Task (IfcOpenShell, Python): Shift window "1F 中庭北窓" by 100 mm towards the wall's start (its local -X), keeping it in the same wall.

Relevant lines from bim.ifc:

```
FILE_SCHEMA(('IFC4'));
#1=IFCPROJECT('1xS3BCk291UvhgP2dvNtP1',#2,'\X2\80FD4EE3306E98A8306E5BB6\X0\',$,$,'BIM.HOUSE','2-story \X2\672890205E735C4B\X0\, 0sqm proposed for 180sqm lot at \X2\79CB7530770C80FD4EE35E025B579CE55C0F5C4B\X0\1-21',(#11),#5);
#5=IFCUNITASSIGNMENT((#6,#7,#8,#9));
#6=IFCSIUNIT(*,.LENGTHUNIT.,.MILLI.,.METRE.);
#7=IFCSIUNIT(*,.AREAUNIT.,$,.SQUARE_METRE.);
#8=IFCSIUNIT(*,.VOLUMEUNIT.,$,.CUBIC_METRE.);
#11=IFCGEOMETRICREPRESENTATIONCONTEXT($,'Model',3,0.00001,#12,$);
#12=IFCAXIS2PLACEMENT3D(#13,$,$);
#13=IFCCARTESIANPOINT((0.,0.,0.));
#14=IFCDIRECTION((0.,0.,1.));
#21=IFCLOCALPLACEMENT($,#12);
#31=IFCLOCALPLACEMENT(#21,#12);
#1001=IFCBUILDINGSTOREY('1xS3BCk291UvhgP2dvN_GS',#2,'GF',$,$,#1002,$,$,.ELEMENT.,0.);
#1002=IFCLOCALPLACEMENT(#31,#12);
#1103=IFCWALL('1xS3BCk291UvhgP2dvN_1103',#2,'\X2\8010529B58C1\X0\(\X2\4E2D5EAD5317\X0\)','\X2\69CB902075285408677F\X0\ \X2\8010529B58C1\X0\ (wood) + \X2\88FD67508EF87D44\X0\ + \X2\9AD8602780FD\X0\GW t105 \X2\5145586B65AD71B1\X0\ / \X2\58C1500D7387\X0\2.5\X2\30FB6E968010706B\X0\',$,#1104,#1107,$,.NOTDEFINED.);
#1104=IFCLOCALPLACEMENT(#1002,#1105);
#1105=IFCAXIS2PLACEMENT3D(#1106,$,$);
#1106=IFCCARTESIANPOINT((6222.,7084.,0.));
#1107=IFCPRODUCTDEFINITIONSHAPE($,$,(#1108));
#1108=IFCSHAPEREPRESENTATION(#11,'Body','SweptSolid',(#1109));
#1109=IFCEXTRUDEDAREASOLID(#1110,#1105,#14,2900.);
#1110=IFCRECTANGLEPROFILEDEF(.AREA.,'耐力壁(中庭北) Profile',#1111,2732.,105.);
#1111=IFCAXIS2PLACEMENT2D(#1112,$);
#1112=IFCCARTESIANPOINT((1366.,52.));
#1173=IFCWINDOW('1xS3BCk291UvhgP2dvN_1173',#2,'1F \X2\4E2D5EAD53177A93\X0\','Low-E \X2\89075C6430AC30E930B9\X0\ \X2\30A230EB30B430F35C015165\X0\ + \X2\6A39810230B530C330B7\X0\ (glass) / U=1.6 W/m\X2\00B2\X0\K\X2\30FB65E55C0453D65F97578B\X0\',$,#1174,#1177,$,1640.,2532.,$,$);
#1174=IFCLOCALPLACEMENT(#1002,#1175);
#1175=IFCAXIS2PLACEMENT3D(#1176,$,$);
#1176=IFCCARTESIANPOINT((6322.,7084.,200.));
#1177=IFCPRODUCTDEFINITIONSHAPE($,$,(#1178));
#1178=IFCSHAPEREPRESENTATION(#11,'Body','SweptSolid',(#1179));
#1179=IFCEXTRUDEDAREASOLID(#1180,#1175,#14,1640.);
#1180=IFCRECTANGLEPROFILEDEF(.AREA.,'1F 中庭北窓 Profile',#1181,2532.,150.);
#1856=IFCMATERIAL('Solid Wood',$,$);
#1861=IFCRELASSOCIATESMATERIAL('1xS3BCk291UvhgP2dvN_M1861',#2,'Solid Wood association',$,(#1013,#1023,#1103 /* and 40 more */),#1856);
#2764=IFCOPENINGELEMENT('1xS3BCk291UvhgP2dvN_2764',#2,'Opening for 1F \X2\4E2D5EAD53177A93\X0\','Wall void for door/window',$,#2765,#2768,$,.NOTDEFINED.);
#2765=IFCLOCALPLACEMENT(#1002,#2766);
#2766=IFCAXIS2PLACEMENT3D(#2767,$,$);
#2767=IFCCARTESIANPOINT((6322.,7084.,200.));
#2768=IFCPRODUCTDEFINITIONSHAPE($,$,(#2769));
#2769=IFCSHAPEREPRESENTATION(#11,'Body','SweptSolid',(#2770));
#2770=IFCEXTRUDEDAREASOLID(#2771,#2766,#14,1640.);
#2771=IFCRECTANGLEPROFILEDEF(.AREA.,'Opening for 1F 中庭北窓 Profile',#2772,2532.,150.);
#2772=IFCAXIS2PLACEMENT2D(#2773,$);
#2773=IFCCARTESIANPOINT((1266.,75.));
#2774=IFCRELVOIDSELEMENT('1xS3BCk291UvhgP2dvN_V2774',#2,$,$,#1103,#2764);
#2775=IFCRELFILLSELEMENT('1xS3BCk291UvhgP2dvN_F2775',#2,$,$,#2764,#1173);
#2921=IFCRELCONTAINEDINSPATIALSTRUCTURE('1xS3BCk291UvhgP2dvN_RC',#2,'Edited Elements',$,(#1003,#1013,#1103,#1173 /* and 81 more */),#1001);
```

```python
import ifcopenshell
import ifcopenshell.api.geometry
import ifcopenshell.util.placement

model = ifcopenshell.open("bim.ifc")

window = model.by_id(1173)
opening = window.FillsVoids[0].RelatingOpeningElement
wall = opening.VoidsElements[0].RelatingBuildingElement

wall_matrix = ifcopenshell.util.placement.get_local_placement(wall.ObjectPlacement)
shift = wall_matrix[:3, 0] * -100.0
before = ifcopenshell.util.placement.get_local_placement(window.ObjectPlacement)[:3, 3].copy()

# The window is not placed relative to its opening, so move both.
for product in (opening, window):
    matrix = ifcopenshell.util.placement.get_local_placement(product.ObjectPlacement)
    matrix[:3, 3] += shift
    ifcopenshell.api.geometry.edit_object_placement(model, product=product, matrix=matrix, is_si=False)

after = ifcopenshell.util.placement.get_local_placement(window.ObjectPlacement)[:3, 3]
print("window moved by", (after - before).round(3) + 0.0)

model.write("bim_rev.ifc")
```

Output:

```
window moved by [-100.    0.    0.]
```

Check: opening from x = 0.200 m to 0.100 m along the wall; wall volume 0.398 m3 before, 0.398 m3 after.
